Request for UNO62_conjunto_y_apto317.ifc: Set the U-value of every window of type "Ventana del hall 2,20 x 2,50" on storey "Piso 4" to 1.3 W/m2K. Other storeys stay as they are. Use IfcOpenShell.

First a look at what the model holds.

```python
import ifcopenshell
import ifcopenshell.util.element

model = ifcopenshell.open("UNO62_conjunto_y_apto317.ifc")
print(model.schema)
storey = next(s for s in model.by_type("IfcBuildingStorey") if s.Name == "Piso 4")
windows = [e for e in ifcopenshell.util.element.get_decomposition(storey) if e.is_a("IfcWindow")]
seen = {}
for e in windows:
    element_type = ifcopenshell.util.element.get_type(e)
    key = (element_type.Name if element_type != e and element_type else None, ifcopenshell.util.element.get_pset(e, "Pset_WindowCommon", "ThermalTransmittance"))
    seen[key] = seen.get(key, 0) + 1
for (name, value), count in sorted(seen.items(), key=str):
    print(count, "x", name, "|", value)
```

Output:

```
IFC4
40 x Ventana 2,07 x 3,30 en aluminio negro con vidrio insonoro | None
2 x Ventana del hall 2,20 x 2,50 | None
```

```python
import ifcopenshell
import ifcopenshell.api.pset
import ifcopenshell.util.element

model = ifcopenshell.open("UNO62_conjunto_y_apto317.ifc")

storey = next(s for s in model.by_type("IfcBuildingStorey") if s.Name == "Piso 4")
windows = [e for e in ifcopenshell.util.element.get_decomposition(storey) if e.is_a("IfcWindow")]

count = 0
for e in windows:
    element_type = ifcopenshell.util.element.get_type(e)
    if element_type in (None, e) or element_type.Name != "Ventana del hall 2,20 x 2,50":
        continue
    found = ifcopenshell.util.element.get_pset(e, "Pset_WindowCommon", should_inherit=False)
    if found:
        pset = model.by_id(found["id"])
        if len(ifcopenshell.util.element.get_elements_by_pset(pset)) > 1:
            pset = ifcopenshell.api.pset.unshare_pset(model, products=[e], pset=pset)[0]
    else:
        pset = ifcopenshell.api.pset.add_pset(model, product=e, name="Pset_WindowCommon")
    ifcopenshell.api.pset.edit_pset(model, pset=pset, properties={"ThermalTransmittance": 1.3})
    count += 1

print(count, "windows updated")

model.write("UNO62_conjunto_y_apto317_updated.ifc")
```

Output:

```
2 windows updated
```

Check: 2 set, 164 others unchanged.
